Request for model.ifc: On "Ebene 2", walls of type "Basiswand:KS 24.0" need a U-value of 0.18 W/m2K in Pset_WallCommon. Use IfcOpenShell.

First a look at what the model holds.

```python
import ifcopenshell
import ifcopenshell.util.element

model = ifcopenshell.open("model.ifc")
print(model.schema)
storey = next(s for s in model.by_type("IfcBuildingStorey") if s.Name == "Ebene 2")
walls = [e for e in ifcopenshell.util.element.get_decomposition(storey) if e.is_a("IfcWall")]
seen = {}
for e in walls:
    element_type = ifcopenshell.util.element.get_type(e)
    key = (element_type.Name if element_type != e and element_type else None, ifcopenshell.util.element.get_pset(e, "Pset_WallCommon", "ThermalTransmittance"))
    seen[key] = seen.get(key, 0) + 1
for (name, value), count in sorted(seen.items(), key=str):
    print(count, "x", name, "|", value)
```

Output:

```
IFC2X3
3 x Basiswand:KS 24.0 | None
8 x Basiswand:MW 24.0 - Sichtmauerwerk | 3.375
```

```python
import ifcopenshell
import ifcopenshell.api.pset
import ifcopenshell.util.element

model = ifcopenshell.open("model.ifc")

storey = next(s for s in model.by_type("IfcBuildingStorey") if s.Name == "Ebene 2")
walls = [e for e in ifcopenshell.util.element.get_decomposition(storey) if e.is_a("IfcWall")]

count = 0
for e in walls:
    element_type = ifcopenshell.util.element.get_type(e)
    if element_type in (None, e) or element_type.Name != "Basiswand:KS 24.0":
        continue
    # add_pset returns the element's existing set when there is one.
    pset = ifcopenshell.api.pset.add_pset(model, product=e, name="Pset_WallCommon")
    ifcopenshell.api.pset.edit_pset(model, pset=pset, properties={"ThermalTransmittance": 0.18})
    count += 1

print(count, "walls updated")

model.write("model_edited.ifc")
```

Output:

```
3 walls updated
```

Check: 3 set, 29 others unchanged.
